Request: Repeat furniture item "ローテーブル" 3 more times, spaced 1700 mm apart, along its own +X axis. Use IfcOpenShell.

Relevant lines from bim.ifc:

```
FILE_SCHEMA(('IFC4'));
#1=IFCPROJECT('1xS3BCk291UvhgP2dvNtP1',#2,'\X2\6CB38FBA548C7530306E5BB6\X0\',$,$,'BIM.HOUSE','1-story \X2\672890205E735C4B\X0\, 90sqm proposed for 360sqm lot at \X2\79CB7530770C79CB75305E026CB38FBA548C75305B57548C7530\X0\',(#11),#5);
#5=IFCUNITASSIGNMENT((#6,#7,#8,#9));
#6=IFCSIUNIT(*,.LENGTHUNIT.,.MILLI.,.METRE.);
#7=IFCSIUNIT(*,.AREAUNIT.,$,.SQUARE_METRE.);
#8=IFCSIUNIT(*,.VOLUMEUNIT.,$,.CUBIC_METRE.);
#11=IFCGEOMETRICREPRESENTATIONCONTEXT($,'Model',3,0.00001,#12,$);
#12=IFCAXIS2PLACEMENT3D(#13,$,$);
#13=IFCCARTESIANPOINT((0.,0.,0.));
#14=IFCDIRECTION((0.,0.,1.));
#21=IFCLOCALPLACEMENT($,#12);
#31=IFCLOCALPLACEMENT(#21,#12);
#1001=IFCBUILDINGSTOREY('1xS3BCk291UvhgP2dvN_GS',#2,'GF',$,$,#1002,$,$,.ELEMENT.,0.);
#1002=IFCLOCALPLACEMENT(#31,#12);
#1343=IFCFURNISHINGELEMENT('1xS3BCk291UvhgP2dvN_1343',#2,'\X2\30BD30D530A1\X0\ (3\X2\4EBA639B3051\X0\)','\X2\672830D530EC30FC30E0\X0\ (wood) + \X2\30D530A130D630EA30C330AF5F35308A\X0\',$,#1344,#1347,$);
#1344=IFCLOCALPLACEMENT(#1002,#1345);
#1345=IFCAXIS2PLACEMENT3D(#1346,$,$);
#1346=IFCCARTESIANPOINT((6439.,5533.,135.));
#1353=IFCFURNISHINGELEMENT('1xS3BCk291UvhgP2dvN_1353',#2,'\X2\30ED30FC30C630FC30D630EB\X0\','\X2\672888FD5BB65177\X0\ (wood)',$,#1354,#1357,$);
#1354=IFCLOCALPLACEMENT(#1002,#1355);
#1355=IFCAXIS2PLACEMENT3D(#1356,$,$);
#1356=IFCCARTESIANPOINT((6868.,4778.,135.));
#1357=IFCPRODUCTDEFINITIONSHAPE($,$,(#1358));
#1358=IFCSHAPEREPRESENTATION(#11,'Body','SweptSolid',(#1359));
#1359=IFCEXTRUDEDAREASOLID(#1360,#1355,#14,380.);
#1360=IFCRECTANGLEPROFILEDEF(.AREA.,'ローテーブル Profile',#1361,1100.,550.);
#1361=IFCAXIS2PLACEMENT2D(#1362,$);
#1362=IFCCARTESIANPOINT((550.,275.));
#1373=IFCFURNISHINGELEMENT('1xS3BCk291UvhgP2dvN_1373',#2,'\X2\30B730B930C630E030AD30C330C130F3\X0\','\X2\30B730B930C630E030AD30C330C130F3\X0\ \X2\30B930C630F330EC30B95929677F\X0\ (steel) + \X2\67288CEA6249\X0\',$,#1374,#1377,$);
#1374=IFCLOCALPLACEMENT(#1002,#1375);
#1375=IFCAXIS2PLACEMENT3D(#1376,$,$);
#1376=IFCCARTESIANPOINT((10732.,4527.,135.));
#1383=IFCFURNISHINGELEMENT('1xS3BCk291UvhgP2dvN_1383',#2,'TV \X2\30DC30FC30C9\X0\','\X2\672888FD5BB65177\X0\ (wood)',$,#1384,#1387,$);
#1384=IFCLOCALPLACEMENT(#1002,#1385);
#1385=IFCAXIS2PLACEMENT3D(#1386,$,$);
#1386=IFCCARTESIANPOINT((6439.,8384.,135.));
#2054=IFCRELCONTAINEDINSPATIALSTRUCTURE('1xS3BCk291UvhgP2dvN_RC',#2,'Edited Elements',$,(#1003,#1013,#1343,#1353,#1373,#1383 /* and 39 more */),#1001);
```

```python
import ifcopenshell
import ifcopenshell.api.geometry
import ifcopenshell.api.root
import ifcopenshell.util.element
import ifcopenshell.util.placement
import ifcopenshell.util.unit

model = ifcopenshell.open("bim.ifc")
unit_scale = ifcopenshell.util.unit.calculate_unit_scale(model)


def reuse_history(source, copy):
    """copy_class also copies each property set's owner history, people and application; keep the originals."""
    for rel in copy.IsDefinedBy:
        if rel.is_a("IfcRelDefinesByProperties") and (history := rel.RelatingPropertyDefinition.OwnerHistory):
            rel.RelatingPropertyDefinition.OwnerHistory = source.OwnerHistory
            ifcopenshell.util.element.remove_deep2(model, history)


source = model.by_guid("1xS3BCk291UvhgP2dvN_1353")
base = ifcopenshell.util.placement.get_local_placement(source.ObjectPlacement)
step = base[:3, 0] * 1.7 / unit_scale

for i in range(1, 4):
    copy = ifcopenshell.api.root.copy_class(model, product=source)
    copy.Representation = ifcopenshell.util.element.copy_deep(
        model, source.Representation, exclude=["IfcGeometricRepresentationContext", "IfcRepresentationMap"]
    )
    reuse_history(source, copy)
    matrix = base.copy()
    matrix[:3, 3] += i * step
    print("added at", matrix[:3, 3].round(3) + 0.0)
    ifcopenshell.api.geometry.edit_object_placement(model, product=copy, matrix=matrix, is_si=False)

model.write("bim_rev.ifc")
```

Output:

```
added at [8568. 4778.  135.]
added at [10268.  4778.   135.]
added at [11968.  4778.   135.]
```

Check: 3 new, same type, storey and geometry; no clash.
